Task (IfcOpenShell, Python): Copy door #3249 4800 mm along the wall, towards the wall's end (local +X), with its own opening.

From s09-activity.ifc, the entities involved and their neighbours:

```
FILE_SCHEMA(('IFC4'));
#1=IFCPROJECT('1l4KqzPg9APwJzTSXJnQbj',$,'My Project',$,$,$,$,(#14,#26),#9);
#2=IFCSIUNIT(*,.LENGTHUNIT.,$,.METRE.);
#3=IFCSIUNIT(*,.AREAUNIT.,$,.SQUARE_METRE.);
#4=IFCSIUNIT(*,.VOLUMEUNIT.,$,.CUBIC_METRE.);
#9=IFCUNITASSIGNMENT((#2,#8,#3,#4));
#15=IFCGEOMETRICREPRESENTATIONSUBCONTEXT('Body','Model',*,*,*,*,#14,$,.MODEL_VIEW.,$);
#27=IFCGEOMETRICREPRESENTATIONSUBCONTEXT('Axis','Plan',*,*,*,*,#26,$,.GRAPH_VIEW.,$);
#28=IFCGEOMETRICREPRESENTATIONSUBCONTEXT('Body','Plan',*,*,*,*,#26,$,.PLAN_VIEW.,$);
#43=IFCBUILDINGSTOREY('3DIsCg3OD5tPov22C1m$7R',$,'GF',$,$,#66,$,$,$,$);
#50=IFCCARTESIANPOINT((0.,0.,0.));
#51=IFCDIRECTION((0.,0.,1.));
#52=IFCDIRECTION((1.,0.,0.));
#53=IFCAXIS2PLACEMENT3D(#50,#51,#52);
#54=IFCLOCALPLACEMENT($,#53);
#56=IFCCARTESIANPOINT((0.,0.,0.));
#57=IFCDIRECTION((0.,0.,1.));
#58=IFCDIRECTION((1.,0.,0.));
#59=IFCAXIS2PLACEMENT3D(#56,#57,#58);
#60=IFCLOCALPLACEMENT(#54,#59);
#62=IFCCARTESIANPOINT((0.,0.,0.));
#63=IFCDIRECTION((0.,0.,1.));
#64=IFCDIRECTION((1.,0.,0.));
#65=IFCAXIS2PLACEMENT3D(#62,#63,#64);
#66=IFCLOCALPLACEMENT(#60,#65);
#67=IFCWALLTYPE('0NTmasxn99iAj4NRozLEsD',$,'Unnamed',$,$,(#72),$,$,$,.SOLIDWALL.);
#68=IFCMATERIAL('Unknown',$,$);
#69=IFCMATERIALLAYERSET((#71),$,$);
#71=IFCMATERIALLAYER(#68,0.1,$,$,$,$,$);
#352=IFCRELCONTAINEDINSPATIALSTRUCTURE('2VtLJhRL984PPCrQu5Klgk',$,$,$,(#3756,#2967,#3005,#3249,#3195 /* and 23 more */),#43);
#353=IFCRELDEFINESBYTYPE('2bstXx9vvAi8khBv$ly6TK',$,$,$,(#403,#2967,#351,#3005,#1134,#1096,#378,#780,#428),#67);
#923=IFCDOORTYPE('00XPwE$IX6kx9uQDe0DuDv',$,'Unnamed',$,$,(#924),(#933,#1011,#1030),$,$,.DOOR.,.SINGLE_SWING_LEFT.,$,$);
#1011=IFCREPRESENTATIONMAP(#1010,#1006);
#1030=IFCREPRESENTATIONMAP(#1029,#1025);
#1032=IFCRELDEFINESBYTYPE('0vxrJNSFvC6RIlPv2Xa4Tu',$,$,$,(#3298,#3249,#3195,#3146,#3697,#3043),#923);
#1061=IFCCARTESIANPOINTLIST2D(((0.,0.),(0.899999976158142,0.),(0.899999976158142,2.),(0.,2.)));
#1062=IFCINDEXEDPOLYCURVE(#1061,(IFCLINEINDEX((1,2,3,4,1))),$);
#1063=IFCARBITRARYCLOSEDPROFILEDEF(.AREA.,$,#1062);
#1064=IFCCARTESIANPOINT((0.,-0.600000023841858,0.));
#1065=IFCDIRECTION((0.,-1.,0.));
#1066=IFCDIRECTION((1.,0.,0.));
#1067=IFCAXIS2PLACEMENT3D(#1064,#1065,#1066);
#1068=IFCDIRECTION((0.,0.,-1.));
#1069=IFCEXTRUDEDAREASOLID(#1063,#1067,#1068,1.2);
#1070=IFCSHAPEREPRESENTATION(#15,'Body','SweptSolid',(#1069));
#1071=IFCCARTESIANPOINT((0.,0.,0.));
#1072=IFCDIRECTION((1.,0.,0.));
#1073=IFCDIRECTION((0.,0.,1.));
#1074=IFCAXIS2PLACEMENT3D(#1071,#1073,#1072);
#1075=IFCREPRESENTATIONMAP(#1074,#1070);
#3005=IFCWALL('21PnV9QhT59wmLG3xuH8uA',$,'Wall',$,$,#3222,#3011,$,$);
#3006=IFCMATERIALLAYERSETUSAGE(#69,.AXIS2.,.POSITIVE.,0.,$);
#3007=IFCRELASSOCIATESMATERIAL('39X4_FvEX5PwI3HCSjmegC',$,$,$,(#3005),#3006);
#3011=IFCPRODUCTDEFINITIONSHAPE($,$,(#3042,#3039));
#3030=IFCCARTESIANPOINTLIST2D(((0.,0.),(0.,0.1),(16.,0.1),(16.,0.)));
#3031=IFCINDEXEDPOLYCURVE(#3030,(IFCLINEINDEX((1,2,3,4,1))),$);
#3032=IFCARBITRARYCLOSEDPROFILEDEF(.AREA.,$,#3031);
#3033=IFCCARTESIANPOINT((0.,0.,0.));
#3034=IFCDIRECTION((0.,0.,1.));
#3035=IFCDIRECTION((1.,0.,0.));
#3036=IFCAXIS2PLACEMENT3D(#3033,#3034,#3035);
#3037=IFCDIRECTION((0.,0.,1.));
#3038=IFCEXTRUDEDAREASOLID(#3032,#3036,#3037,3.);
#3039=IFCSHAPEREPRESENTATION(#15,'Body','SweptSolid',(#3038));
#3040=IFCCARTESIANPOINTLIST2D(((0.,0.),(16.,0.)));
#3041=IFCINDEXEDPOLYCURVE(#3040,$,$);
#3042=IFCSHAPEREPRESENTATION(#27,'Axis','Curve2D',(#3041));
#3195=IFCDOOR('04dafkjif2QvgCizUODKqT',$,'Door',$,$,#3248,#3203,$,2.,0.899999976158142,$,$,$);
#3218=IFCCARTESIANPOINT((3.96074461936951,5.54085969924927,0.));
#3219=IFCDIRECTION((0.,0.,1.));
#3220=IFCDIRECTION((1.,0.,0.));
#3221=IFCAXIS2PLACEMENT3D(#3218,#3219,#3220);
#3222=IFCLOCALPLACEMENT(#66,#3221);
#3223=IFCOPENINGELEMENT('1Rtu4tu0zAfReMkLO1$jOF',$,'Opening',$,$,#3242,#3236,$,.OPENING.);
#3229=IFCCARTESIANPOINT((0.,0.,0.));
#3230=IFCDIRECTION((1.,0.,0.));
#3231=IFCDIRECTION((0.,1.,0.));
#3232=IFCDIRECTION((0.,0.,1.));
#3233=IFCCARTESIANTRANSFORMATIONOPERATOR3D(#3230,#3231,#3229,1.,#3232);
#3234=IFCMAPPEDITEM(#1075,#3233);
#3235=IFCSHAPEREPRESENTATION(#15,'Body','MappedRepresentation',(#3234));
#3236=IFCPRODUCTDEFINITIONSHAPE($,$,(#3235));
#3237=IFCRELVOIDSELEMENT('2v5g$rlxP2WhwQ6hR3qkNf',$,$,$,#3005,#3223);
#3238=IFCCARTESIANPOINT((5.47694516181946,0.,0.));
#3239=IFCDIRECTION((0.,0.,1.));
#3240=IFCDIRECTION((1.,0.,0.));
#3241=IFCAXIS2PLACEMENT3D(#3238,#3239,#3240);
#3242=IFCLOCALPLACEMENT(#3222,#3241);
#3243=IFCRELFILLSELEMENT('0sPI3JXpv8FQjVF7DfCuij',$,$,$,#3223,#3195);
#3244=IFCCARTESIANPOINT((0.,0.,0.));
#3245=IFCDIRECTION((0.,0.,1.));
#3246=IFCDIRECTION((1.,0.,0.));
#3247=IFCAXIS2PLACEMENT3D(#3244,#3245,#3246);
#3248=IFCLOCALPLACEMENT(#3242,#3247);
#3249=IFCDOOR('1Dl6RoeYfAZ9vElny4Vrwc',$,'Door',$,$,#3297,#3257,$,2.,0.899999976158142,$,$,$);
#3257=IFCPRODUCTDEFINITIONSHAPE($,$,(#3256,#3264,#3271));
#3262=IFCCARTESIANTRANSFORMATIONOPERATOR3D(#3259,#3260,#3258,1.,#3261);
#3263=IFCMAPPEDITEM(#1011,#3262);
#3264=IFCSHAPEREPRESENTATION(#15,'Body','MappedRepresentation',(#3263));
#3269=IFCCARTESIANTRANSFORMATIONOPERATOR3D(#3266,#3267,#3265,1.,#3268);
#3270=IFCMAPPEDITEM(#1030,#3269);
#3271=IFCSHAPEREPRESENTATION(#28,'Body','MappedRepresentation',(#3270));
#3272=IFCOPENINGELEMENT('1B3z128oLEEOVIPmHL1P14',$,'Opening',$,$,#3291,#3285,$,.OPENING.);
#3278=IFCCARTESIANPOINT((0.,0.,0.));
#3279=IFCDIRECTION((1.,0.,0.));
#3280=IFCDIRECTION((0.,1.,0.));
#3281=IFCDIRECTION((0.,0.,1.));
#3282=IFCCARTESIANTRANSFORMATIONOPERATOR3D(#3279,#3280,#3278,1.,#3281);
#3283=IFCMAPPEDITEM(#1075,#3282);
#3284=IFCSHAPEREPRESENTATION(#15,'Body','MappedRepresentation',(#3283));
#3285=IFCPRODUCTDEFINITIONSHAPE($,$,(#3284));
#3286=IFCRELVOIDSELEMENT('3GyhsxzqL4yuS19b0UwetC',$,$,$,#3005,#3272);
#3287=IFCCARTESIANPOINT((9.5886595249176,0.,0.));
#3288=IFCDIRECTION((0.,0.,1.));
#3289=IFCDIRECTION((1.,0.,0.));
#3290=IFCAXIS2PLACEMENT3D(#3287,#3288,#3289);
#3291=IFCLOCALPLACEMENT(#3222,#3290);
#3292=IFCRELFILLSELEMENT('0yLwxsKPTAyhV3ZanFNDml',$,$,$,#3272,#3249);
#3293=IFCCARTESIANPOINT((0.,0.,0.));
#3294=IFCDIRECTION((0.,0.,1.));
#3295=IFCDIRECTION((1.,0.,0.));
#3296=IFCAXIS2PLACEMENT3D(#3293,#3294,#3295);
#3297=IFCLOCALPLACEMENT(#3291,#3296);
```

```python
import ifcopenshell
import ifcopenshell.api.feature
import ifcopenshell.api.geometry
import ifcopenshell.api.root
import ifcopenshell.geom
import ifcopenshell.util.element
import ifcopenshell.util.placement
import ifcopenshell.util.shape

model = ifcopenshell.open("s09-activity.ifc")
settings = ifcopenshell.geom.settings()


def volume(element):
    """Net volume in cubic metres, openings subtracted."""
    shape = ifcopenshell.geom.create_shape(settings, element)
    return ifcopenshell.util.shape.get_volume(shape.geometry)


door = model.by_guid("1Dl6RoeYfAZ9vElny4Vrwc")
opening = door.FillsVoids[0].RelatingOpeningElement
wall = opening.VoidsElements[0].RelatingBuildingElement
before = volume(wall)
shift = ifcopenshell.util.placement.get_local_placement(wall.ObjectPlacement)[:3, 0] * 4.8

# copy_class copies the void relationship, type, container and properties, but no geometry.
new_opening = ifcopenshell.api.root.copy_class(model, product=opening)
new_opening.Representation = ifcopenshell.util.element.copy_deep(
    model, opening.Representation, exclude=["IfcGeometricRepresentationContext", "IfcRepresentationMap"]
)
new_door = ifcopenshell.api.root.copy_class(model, product=door)
new_door.Representation = ifcopenshell.util.element.copy_deep(
    model, door.Representation, exclude=["IfcGeometricRepresentationContext", "IfcRepresentationMap"]
)
ifcopenshell.api.feature.add_filling(model, opening=new_opening, element=new_door)

for old, new in ((opening, new_opening), (door, new_door)):
    matrix = ifcopenshell.util.placement.get_local_placement(old.ObjectPlacement)
    matrix[:3, 3] += shift
    ifcopenshell.api.geometry.edit_object_placement(model, product=new, matrix=matrix, is_si=False)

after = volume(wall)

print(f"wall volume {before:.3f} -> {after:.3f} m3")

model.write("s09-activity-out.ifc")
```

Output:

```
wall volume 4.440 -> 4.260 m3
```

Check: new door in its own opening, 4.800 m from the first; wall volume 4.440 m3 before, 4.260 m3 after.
